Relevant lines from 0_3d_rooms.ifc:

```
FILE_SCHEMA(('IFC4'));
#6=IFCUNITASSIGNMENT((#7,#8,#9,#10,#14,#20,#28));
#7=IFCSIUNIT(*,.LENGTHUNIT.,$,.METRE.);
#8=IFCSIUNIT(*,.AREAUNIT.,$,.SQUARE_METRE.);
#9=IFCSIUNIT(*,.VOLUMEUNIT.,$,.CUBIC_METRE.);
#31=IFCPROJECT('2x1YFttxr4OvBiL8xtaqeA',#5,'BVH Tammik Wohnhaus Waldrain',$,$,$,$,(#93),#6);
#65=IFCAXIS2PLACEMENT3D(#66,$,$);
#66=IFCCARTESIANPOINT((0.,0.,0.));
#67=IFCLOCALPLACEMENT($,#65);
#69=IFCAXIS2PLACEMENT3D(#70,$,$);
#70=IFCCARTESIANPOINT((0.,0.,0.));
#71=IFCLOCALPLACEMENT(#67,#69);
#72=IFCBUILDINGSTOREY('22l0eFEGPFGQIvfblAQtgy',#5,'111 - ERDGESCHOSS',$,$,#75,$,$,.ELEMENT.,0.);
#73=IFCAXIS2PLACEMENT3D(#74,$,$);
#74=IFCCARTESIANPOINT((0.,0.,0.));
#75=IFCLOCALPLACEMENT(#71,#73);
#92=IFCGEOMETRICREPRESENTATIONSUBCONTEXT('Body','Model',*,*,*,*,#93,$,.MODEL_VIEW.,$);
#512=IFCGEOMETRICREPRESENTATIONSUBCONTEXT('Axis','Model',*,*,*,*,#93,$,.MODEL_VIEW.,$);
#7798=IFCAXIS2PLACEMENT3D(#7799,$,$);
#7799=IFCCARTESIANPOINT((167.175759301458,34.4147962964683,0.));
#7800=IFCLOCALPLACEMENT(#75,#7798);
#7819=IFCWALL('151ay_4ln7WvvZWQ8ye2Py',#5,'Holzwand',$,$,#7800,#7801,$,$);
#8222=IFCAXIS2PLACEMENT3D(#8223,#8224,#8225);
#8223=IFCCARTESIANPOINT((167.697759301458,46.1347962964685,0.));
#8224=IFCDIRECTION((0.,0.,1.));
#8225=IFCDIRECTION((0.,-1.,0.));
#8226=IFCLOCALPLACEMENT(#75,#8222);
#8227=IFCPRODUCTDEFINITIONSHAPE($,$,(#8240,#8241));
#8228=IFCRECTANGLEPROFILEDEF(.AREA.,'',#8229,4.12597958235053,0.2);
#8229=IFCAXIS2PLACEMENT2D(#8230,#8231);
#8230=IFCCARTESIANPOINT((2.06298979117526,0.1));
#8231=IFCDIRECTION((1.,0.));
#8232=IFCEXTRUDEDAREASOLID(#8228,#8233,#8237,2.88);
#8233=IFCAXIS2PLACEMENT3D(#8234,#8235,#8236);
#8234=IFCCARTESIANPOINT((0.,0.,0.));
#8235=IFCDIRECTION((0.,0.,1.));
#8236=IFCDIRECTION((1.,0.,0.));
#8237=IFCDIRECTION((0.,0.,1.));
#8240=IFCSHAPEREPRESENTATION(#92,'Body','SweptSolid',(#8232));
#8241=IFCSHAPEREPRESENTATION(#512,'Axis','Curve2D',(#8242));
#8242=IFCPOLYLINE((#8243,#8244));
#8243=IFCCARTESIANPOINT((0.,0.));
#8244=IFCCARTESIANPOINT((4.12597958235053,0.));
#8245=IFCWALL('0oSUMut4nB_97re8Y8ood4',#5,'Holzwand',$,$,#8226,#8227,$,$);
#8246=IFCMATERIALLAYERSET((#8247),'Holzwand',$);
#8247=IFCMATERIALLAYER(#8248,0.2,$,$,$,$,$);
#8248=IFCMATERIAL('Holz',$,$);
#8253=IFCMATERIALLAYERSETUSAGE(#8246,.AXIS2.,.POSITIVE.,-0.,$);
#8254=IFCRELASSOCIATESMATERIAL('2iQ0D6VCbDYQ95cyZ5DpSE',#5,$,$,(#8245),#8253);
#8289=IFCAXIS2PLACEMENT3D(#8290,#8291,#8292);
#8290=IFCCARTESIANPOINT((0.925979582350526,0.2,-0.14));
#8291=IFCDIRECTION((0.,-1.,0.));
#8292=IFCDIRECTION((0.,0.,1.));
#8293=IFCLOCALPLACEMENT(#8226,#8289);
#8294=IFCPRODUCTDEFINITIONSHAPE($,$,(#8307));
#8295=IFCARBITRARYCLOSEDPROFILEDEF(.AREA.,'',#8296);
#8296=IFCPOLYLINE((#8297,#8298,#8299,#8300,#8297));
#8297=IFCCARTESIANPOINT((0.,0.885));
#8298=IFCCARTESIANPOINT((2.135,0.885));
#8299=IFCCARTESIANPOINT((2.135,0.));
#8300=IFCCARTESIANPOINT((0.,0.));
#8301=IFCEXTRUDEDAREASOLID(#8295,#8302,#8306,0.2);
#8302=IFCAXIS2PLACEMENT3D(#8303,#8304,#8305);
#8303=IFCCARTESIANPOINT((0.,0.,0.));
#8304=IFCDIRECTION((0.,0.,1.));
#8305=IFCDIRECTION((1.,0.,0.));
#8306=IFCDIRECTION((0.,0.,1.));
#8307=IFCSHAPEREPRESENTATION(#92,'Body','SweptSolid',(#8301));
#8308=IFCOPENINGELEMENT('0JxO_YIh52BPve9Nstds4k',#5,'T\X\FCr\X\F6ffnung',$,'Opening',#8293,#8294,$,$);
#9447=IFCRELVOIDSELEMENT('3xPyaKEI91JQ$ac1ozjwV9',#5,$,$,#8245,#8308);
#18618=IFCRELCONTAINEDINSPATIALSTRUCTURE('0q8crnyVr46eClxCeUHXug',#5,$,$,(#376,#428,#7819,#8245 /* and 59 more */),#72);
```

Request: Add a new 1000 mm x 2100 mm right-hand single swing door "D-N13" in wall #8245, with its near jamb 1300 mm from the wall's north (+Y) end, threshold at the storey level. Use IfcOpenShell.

```python
import numpy as np
import ifcopenshell
import ifcopenshell.api.feature
import ifcopenshell.api.geometry
import ifcopenshell.api.root
import ifcopenshell.api.spatial
import ifcopenshell.geom
import ifcopenshell.util.element
import ifcopenshell.util.placement
import ifcopenshell.util.representation
import ifcopenshell.util.shape
import ifcopenshell.util.unit

model = ifcopenshell.open("0_3d_rooms.ifc")
unit_scale = ifcopenshell.util.unit.calculate_unit_scale(model)
settings = ifcopenshell.geom.settings()


def volume(element):
    """Net volume in cubic metres, openings subtracted."""
    shape = ifcopenshell.geom.create_shape(settings, element)
    return ifcopenshell.util.shape.get_volume(shape.geometry)


wall = model.by_guid("0oSUMut4nB_97re8Y8ood4")
storey = ifcopenshell.util.element.get_container(wall, ifc_class="IfcBuildingStorey")
context = ifcopenshell.util.representation.get_context(model, "Model", "Body", "MODEL_VIEW")
before = volume(wall)

width, height, from_end, sill = 1, 2.1, 1.3, 0.0  # metres

# The wall runs along its own X axis, and the end named is its -X end.
wall_shape = ifcopenshell.geom.create_shape(settings, wall)
x, y, z = ifcopenshell.util.shape.get_vertices(wall_shape.geometry).T
start = x.min() + from_end
face, thickness = float(y.min()), float(y.max() - y.min())
wall_matrix = ifcopenshell.util.placement.get_local_placement(wall.ObjectPlacement)
level = ifcopenshell.util.placement.get_local_placement(storey.ObjectPlacement)[2, 3]


def in_wall(x, y):
    """Placement at x, y metres in the wall's axes, at sill height."""
    matrix = wall_matrix.copy()
    matrix[:, 3] = wall_matrix @ np.array([x / unit_scale, y / unit_scale, 0.0, 1.0])
    matrix[2, 3] = level + sill / unit_scale
    return matrix


# Opening: a box that overshoots both wall faces by 50 mm.
opening = ifcopenshell.api.root.create_entity(model, ifc_class="IfcOpeningElement", predefined_type="OPENING")
box = ifcopenshell.api.geometry.add_wall_representation(
    model, context=context, length=width, height=height, thickness=thickness + 0.1
)
ifcopenshell.api.geometry.assign_representation(model, product=opening, representation=box)
ifcopenshell.api.geometry.edit_object_placement(model, product=opening, matrix=in_wall(start, face - 0.05), is_si=False)
ifcopenshell.api.feature.add_feature(model, feature=opening, element=wall)

door = ifcopenshell.api.root.create_entity(model, ifc_class="IfcDoor", name="D-N13", predefined_type="DOOR")
door.OverallWidth, door.OverallHeight = width / unit_scale, height / unit_scale
door.OperationType = "SINGLE_SWING_RIGHT"
body = ifcopenshell.api.geometry.add_door_representation(
    model,
    context=context,
    overall_width=door.OverallWidth,
    overall_height=door.OverallHeight,
    operation_type="SINGLE_SWING_RIGHT",
    lining_properties={"LiningDepth": thickness / unit_scale, "ThresholdDepth": thickness / unit_scale},
)
ifcopenshell.api.geometry.assign_representation(model, product=door, representation=body)
ifcopenshell.api.spatial.assign_container(model, products=[door], relating_structure=storey)
ifcopenshell.api.feature.add_filling(model, opening=opening, element=door)

# The lining spans the wall, so the door starts at the wall face.
ifcopenshell.api.geometry.edit_object_placement(model, product=door, matrix=in_wall(start, face), is_si=False)

after = volume(wall)

print(f"wall volume {before:.3f} -> {after:.3f} m3")

model.write("0_3d_rooms_v2.ifc")
```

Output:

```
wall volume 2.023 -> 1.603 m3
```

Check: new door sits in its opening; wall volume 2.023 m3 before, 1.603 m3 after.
